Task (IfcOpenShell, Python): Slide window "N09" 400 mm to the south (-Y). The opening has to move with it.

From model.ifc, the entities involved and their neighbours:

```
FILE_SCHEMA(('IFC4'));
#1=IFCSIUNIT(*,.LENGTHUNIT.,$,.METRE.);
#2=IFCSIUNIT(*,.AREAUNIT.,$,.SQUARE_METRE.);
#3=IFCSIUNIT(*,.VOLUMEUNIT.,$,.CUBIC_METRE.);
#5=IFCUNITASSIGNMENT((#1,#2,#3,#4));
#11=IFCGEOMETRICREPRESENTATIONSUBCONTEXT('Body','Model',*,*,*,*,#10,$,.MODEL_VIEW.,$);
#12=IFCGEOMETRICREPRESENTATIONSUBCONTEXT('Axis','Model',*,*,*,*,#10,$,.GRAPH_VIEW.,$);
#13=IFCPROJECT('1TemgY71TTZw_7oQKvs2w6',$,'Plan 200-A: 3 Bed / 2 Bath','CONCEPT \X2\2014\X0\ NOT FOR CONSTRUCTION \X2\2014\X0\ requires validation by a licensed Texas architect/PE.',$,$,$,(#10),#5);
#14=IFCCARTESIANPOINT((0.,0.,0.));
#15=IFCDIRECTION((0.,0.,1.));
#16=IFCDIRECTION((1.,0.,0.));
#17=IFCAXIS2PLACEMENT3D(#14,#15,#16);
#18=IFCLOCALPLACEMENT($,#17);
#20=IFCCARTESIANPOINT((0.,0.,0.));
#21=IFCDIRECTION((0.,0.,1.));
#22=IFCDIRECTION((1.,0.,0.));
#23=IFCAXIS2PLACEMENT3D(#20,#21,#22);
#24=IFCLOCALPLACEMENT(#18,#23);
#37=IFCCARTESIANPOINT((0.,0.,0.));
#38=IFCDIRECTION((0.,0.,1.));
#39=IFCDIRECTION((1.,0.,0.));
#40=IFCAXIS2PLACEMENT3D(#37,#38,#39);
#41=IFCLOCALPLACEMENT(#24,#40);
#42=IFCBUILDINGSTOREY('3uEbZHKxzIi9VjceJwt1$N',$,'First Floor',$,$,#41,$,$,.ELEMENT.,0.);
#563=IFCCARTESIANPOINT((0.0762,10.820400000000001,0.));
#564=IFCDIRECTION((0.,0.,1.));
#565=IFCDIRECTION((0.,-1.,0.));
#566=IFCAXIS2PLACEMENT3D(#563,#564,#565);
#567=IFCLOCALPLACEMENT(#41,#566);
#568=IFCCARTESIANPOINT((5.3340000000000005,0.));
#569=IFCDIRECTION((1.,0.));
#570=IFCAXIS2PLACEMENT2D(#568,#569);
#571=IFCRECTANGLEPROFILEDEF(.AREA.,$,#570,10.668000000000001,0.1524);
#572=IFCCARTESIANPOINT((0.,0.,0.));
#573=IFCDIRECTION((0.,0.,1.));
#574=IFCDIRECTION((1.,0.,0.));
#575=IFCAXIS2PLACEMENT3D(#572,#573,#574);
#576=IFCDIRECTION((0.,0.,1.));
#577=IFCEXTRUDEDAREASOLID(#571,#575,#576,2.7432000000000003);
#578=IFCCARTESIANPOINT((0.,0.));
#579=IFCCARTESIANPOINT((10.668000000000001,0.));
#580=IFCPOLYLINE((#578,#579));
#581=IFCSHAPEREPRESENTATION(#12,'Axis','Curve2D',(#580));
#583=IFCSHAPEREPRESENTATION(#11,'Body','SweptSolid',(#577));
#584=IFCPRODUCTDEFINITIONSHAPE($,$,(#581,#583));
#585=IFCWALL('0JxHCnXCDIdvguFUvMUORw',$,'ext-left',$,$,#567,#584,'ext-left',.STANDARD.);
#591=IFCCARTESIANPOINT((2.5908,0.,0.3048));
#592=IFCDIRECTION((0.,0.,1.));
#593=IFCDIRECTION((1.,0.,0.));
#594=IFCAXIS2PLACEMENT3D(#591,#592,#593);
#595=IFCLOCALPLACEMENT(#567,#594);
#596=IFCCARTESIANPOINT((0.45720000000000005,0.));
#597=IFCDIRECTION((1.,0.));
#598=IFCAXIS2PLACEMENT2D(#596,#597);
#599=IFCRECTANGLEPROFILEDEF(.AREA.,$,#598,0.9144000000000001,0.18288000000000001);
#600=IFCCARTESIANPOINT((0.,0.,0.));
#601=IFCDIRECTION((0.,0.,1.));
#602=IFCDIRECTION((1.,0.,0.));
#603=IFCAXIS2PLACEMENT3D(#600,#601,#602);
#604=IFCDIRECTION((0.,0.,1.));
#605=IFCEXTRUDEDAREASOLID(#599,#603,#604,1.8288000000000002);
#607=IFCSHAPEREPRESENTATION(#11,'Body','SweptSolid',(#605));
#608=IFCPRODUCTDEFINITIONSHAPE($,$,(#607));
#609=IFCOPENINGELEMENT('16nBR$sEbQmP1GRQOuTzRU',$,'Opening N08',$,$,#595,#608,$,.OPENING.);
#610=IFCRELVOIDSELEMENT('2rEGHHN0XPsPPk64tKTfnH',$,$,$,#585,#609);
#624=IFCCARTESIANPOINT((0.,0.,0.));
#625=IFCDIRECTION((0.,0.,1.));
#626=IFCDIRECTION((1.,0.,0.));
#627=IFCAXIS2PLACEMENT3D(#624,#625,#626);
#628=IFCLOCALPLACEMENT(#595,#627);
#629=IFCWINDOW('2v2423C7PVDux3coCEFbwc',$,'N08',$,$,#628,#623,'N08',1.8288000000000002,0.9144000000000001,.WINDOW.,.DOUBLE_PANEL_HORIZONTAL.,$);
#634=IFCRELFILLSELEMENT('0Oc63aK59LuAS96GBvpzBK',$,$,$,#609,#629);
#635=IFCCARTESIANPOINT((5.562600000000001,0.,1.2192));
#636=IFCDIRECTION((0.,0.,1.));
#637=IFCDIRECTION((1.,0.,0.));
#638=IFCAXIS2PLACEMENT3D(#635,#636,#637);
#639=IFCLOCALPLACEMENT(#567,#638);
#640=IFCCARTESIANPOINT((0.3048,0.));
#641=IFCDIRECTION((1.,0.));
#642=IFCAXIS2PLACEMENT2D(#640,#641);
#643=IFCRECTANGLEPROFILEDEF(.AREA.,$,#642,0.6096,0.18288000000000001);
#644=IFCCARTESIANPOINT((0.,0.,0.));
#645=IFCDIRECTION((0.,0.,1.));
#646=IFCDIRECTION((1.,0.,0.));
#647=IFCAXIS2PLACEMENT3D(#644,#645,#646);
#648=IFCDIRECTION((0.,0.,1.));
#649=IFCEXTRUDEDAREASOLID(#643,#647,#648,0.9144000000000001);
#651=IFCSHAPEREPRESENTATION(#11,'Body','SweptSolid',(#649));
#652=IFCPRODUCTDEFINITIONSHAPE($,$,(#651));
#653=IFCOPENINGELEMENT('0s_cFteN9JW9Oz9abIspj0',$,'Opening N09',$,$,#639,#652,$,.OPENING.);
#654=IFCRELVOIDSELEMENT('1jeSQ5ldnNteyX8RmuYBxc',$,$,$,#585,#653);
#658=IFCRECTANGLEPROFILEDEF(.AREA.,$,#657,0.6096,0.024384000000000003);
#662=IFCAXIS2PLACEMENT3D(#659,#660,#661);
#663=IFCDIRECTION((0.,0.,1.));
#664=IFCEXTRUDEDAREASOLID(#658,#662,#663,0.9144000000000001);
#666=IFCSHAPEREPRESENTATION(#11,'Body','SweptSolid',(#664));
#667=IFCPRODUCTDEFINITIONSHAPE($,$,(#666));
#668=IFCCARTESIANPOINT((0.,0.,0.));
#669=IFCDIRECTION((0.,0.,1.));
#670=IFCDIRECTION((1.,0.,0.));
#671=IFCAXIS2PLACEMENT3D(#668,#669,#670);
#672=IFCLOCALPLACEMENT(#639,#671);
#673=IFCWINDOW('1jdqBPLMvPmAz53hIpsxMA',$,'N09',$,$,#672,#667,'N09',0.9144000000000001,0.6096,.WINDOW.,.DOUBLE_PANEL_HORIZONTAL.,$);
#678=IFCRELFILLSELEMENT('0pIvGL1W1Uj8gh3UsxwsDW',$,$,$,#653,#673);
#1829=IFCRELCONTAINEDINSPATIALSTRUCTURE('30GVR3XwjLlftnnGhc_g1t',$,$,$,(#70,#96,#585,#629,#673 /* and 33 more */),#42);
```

```python
import ifcopenshell
import ifcopenshell.api.geometry
import ifcopenshell.util.placement
import ifcopenshell.util.unit

model = ifcopenshell.open("model.ifc")
unit_scale = ifcopenshell.util.unit.calculate_unit_scale(model)

window = model.by_id(673)
opening = window.FillsVoids[0].RelatingOpeningElement
wall = opening.VoidsElements[0].RelatingBuildingElement

wall_matrix = ifcopenshell.util.placement.get_local_placement(wall.ObjectPlacement)
shift = wall_matrix[:3, 0] * 0.4 / unit_scale
before = ifcopenshell.util.placement.get_local_placement(window.ObjectPlacement)[:3, 3].copy()

# The window is placed relative to its opening, so it follows when the opening moves.
matrix = ifcopenshell.util.placement.get_local_placement(opening.ObjectPlacement)
matrix[:3, 3] += shift
ifcopenshell.api.geometry.edit_object_placement(
    model, product=opening, matrix=matrix, is_si=False, should_transform_children=True
)

after = ifcopenshell.util.placement.get_local_placement(window.ObjectPlacement)[:3, 3]
print("window moved by", (after - before).round(3) + 0.0)

model.write("model_v2.ifc")
```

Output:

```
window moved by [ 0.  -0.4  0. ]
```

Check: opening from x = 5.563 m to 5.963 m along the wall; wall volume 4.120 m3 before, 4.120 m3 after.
